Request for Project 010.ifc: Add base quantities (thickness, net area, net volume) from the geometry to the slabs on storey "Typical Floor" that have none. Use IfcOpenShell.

First a look at what the model holds.

```python
import ifcopenshell
import ifcopenshell.util.element
import ifcopenshell.util.unit

model = ifcopenshell.open("Project 010.ifc")
print(model.schema)
for unit_type in ("LENGTHUNIT", "AREAUNIT", "VOLUMEUNIT"):
    print(unit_type, ifcopenshell.util.unit.calculate_unit_scale(model, unit_type))
storey = next(s for s in model.by_type("IfcBuildingStorey") if s.Name == "Typical Floor")
slabs = [e for e in ifcopenshell.util.element.get_decomposition(storey) if e.is_a("IfcSlab")]
for e in sorted(slabs, key=lambda e: e.id()):
    print(e.id(), e.is_a(), e.Name, list(ifcopenshell.util.element.get_psets(e, qtos_only=True)), sep=" | ")
```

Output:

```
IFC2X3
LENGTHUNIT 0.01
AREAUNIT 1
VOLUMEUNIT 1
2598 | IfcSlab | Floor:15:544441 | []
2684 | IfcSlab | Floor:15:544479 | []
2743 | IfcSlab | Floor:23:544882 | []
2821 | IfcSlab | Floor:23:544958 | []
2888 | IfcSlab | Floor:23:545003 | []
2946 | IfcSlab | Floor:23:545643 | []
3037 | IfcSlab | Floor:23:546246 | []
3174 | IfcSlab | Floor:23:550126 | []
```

```python
import ifcopenshell
import ifcopenshell.api.pset
import ifcopenshell.geom
import ifcopenshell.util.element
import ifcopenshell.util.shape
import ifcopenshell.util.unit

model = ifcopenshell.open("Project 010.ifc")
unit_scale = ifcopenshell.util.unit.calculate_unit_scale(model)
area_scale = ifcopenshell.util.unit.calculate_unit_scale(model, "AREAUNIT")
volume_scale = ifcopenshell.util.unit.calculate_unit_scale(model, "VOLUMEUNIT")
settings = ifcopenshell.geom.settings()

storey = next(s for s in model.by_type("IfcBuildingStorey") if s.Name == "Typical Floor")
slabs = [e for e in ifcopenshell.util.element.get_decomposition(storey) if e.is_a("IfcSlab")]

for e in sorted(slabs, key=lambda e: e.id()):
    if ifcopenshell.util.element.get_psets(e, qtos_only=True, should_inherit=False):
        continue
    # Geometry comes back in metres, in the element's own axes.
    shape = ifcopenshell.geom.create_shape(settings, e)
    values = {
        "Width": ifcopenshell.util.shape.get_z(shape.geometry) / unit_scale,
        "NetArea": ifcopenshell.util.shape.get_footprint_area(shape.geometry) / area_scale,
        "NetVolume": ifcopenshell.util.shape.get_volume(shape.geometry) / volume_scale,
    }
    qto = ifcopenshell.api.pset.add_qto(model, product=e, name="BaseQuantities")
    ifcopenshell.api.pset.edit_qto(model, qto=qto, properties=values)
    print(e.id(), {k: round(v, 3) for k, v in values.items()})

model.write("Project 010_rev.ifc")
```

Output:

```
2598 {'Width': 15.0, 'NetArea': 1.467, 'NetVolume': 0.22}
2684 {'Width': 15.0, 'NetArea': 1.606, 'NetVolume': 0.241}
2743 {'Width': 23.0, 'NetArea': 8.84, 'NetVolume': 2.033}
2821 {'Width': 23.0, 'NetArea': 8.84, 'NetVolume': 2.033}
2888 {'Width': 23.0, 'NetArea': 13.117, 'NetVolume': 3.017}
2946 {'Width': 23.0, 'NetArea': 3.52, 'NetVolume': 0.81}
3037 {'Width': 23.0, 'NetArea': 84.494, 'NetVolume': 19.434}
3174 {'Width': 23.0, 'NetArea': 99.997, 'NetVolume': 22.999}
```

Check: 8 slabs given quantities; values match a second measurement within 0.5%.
